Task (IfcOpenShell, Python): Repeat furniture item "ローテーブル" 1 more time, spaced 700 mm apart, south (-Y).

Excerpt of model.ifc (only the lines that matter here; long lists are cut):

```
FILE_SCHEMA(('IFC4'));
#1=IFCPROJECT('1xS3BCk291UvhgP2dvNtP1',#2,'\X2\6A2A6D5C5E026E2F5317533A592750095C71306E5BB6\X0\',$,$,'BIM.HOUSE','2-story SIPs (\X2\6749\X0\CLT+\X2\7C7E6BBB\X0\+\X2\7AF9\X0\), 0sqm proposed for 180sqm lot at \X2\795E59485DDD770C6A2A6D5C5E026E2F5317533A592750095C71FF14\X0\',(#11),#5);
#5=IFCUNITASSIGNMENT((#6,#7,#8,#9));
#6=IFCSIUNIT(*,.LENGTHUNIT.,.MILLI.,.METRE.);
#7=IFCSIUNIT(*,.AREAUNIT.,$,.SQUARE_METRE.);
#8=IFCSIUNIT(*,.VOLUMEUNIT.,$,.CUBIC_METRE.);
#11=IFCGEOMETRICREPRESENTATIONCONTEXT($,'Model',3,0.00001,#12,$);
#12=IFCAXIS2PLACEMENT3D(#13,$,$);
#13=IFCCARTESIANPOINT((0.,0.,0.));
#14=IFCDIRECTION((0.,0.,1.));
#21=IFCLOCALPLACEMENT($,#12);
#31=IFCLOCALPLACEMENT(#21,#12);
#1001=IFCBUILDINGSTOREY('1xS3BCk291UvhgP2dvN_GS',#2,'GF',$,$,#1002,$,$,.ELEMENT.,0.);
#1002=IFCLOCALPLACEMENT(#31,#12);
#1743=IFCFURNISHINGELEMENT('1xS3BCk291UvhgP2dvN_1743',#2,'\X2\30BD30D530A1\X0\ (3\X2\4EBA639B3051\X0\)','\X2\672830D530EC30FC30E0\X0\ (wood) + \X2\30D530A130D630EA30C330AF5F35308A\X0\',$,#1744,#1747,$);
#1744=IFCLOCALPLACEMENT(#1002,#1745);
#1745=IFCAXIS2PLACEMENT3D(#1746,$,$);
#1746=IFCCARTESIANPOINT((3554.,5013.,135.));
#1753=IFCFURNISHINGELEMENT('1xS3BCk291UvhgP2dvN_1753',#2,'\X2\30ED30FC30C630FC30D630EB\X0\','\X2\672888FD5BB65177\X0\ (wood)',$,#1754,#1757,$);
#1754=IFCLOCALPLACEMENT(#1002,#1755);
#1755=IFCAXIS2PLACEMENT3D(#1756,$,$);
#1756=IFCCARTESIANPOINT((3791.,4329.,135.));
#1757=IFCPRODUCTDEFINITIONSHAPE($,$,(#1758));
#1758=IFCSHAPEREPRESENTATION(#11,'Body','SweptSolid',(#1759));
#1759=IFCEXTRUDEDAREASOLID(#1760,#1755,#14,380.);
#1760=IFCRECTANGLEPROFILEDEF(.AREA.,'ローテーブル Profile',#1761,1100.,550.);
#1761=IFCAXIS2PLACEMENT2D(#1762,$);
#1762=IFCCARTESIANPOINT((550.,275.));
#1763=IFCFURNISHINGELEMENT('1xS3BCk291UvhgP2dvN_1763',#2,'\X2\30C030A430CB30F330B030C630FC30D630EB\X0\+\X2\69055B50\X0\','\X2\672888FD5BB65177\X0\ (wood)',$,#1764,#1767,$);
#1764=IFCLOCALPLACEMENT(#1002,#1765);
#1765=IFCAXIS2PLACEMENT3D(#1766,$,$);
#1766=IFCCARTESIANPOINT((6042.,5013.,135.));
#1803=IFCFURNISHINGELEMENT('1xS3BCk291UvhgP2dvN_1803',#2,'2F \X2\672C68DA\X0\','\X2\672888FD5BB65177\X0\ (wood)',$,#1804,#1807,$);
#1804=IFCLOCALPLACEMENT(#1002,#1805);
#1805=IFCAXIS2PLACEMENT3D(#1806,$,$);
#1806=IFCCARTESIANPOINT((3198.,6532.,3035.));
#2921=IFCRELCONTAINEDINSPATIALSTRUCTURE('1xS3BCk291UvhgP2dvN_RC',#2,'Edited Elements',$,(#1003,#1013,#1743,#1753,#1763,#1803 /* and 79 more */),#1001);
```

```python
import numpy as np
import ifcopenshell
import ifcopenshell.api.geometry
import ifcopenshell.api.root
import ifcopenshell.util.element
import ifcopenshell.util.placement
import ifcopenshell.util.unit

model = ifcopenshell.open("model.ifc")
unit_scale = ifcopenshell.util.unit.calculate_unit_scale(model)


def reuse_history(source, copy):
    """copy_class also copies each property set's owner history, people and application; keep the originals."""
    for rel in copy.IsDefinedBy:
        if rel.is_a("IfcRelDefinesByProperties") and (history := rel.RelatingPropertyDefinition.OwnerHistory):
            rel.RelatingPropertyDefinition.OwnerHistory = source.OwnerHistory
            ifcopenshell.util.element.remove_deep2(model, history)


source = model.by_id(1753)
base = ifcopenshell.util.placement.get_local_placement(source.ObjectPlacement)
step = np.array([0.0, -1.0, 0.0]) * 0.7 / unit_scale

for i in range(1, 2):
    copy = ifcopenshell.api.root.copy_class(model, product=source)
    copy.Representation = ifcopenshell.util.element.copy_deep(
        model, source.Representation, exclude=["IfcGeometricRepresentationContext", "IfcRepresentationMap"]
    )
    reuse_history(source, copy)
    matrix = base.copy()
    matrix[:3, 3] += i * step
    print("added at", matrix[:3, 3].round(3) + 0.0)
    ifcopenshell.api.geometry.edit_object_placement(model, product=copy, matrix=matrix, is_si=False)

model.write("model_v2.ifc")
```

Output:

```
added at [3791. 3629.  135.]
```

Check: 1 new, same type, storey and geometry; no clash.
